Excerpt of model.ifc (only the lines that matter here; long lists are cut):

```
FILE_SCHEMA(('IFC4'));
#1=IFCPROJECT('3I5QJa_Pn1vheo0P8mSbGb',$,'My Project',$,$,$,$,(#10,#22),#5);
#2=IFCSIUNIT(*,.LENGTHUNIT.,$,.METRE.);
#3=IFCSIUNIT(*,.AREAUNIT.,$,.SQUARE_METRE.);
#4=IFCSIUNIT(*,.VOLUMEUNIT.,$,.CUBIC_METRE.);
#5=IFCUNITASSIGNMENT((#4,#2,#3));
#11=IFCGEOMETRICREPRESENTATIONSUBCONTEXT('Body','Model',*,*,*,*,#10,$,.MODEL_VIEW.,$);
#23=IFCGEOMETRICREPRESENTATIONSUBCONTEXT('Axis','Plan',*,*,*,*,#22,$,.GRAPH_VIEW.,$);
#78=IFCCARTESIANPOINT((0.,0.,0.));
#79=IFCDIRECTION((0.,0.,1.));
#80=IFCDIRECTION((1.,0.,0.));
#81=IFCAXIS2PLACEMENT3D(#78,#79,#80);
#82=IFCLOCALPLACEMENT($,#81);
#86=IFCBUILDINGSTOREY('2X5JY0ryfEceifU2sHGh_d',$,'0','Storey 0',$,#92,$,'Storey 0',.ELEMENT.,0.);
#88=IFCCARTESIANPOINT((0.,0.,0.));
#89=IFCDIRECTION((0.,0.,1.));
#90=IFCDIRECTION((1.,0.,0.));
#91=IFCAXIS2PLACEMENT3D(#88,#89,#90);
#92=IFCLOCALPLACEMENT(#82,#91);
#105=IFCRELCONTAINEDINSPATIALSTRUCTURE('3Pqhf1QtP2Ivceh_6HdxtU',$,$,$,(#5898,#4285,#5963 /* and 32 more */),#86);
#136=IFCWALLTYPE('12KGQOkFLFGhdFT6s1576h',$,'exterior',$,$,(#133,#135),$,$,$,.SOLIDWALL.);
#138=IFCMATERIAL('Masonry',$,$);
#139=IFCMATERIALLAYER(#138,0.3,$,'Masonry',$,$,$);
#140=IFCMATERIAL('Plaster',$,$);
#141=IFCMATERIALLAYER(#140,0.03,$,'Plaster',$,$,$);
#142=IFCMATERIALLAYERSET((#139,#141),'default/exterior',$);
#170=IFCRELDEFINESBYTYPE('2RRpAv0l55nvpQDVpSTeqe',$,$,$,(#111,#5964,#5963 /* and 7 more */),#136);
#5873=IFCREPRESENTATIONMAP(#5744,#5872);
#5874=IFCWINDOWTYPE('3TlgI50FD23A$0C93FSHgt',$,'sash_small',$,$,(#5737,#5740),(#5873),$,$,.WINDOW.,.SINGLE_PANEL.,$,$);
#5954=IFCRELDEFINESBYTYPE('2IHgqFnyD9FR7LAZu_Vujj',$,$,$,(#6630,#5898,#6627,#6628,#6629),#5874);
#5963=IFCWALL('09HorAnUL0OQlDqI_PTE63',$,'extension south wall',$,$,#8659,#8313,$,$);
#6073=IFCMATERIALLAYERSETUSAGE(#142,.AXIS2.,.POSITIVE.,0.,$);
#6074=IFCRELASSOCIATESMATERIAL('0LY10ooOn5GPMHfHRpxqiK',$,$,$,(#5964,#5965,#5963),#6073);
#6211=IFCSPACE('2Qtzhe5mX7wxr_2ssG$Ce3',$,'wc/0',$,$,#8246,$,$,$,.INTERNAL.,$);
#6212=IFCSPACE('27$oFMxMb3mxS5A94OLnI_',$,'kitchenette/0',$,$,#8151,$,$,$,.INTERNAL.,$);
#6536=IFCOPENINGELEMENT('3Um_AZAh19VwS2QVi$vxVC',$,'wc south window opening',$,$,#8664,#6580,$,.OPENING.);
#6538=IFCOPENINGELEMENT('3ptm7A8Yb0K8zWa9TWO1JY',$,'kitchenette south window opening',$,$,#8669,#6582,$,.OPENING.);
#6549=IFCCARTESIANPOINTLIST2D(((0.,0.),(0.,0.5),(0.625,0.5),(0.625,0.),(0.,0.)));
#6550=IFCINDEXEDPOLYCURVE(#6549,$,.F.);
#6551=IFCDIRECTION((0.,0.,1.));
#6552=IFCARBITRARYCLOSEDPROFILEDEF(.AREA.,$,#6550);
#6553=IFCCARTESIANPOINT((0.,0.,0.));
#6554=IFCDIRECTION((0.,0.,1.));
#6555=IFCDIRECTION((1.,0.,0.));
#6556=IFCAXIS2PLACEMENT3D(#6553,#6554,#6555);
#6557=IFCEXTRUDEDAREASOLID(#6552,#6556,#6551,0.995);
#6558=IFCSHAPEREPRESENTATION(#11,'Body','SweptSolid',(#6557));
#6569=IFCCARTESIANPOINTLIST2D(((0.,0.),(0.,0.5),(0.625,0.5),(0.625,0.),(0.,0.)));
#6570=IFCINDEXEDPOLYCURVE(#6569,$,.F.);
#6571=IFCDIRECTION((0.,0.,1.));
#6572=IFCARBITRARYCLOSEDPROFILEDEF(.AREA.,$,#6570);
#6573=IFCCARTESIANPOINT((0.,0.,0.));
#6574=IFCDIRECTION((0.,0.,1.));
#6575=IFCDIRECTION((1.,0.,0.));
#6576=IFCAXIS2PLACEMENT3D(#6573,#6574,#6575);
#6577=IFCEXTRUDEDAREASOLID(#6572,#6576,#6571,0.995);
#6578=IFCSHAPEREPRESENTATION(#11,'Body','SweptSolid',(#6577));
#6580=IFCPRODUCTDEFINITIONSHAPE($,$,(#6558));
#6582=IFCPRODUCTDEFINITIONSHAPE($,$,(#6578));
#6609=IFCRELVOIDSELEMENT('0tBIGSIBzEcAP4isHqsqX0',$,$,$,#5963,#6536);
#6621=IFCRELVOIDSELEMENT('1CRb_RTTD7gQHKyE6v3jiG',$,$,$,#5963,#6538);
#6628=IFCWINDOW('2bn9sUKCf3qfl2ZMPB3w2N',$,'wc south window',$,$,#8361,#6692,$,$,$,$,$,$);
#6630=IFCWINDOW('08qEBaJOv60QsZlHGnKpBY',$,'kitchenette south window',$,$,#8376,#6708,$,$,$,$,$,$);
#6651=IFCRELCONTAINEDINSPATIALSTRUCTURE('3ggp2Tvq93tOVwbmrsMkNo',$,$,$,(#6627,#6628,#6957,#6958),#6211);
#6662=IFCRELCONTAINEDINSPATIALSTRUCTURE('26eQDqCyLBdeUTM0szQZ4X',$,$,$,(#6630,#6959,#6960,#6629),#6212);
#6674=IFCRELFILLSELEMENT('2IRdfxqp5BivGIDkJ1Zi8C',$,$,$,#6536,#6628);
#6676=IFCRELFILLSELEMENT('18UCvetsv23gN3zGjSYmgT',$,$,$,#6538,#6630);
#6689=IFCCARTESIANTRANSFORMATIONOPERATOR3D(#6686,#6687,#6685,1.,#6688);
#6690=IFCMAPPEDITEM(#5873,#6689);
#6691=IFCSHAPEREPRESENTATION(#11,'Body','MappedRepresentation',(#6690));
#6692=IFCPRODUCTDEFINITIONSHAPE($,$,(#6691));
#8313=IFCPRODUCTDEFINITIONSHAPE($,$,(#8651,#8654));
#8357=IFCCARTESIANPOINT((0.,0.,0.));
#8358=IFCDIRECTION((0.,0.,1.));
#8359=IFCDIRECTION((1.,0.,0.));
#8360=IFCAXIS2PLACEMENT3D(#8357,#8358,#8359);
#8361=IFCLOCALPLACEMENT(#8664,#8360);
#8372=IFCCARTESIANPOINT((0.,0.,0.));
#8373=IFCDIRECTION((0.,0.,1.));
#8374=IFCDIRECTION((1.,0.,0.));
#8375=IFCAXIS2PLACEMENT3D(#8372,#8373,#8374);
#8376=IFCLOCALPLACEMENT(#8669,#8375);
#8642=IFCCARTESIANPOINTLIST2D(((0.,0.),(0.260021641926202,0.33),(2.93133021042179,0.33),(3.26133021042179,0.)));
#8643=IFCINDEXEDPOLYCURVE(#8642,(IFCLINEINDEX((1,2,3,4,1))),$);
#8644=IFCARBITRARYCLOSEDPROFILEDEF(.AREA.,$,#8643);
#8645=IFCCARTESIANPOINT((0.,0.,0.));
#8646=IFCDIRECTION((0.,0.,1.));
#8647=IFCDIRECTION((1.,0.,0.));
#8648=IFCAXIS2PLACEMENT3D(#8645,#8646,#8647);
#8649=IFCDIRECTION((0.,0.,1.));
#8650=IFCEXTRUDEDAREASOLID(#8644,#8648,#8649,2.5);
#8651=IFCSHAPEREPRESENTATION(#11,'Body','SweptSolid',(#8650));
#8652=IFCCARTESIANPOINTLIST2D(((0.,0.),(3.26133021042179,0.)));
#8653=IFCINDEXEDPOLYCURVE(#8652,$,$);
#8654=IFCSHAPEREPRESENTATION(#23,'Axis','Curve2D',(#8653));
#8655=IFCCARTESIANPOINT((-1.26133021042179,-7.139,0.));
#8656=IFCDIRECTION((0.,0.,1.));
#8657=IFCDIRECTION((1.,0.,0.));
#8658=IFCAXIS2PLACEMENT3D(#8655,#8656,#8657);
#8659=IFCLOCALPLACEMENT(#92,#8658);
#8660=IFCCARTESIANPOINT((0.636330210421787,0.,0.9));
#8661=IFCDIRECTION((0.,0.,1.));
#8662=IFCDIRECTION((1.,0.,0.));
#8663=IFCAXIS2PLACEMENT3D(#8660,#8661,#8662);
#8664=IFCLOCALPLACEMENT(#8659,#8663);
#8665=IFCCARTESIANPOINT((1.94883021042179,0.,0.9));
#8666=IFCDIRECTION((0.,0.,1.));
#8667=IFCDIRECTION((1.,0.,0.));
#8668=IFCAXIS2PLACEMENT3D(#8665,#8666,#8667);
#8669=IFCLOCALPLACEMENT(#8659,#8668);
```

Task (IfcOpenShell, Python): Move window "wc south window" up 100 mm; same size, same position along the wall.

```python
import numpy as np
import ifcopenshell
import ifcopenshell.api.geometry
import ifcopenshell.util.placement
import ifcopenshell.util.unit

model = ifcopenshell.open("model.ifc")
unit_scale = ifcopenshell.util.unit.calculate_unit_scale(model)

window = model.by_guid("2bn9sUKCf3qfl2ZMPB3w2N")
opening = window.FillsVoids[0].RelatingOpeningElement
dz = 0.1 / unit_scale

shift = np.array([0.0, 0.0, dz])
# The window is placed relative to its opening, so it follows when the opening moves.
matrix = ifcopenshell.util.placement.get_local_placement(opening.ObjectPlacement)
matrix[:3, 3] += shift
ifcopenshell.api.geometry.edit_object_placement(
    model, product=opening, matrix=matrix, is_si=False, should_transform_children=True
)

print(f"moved by {dz * unit_scale:+.3f} m")

model.write("model_rev.ifc")
```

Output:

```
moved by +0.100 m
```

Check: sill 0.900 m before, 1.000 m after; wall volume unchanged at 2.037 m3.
